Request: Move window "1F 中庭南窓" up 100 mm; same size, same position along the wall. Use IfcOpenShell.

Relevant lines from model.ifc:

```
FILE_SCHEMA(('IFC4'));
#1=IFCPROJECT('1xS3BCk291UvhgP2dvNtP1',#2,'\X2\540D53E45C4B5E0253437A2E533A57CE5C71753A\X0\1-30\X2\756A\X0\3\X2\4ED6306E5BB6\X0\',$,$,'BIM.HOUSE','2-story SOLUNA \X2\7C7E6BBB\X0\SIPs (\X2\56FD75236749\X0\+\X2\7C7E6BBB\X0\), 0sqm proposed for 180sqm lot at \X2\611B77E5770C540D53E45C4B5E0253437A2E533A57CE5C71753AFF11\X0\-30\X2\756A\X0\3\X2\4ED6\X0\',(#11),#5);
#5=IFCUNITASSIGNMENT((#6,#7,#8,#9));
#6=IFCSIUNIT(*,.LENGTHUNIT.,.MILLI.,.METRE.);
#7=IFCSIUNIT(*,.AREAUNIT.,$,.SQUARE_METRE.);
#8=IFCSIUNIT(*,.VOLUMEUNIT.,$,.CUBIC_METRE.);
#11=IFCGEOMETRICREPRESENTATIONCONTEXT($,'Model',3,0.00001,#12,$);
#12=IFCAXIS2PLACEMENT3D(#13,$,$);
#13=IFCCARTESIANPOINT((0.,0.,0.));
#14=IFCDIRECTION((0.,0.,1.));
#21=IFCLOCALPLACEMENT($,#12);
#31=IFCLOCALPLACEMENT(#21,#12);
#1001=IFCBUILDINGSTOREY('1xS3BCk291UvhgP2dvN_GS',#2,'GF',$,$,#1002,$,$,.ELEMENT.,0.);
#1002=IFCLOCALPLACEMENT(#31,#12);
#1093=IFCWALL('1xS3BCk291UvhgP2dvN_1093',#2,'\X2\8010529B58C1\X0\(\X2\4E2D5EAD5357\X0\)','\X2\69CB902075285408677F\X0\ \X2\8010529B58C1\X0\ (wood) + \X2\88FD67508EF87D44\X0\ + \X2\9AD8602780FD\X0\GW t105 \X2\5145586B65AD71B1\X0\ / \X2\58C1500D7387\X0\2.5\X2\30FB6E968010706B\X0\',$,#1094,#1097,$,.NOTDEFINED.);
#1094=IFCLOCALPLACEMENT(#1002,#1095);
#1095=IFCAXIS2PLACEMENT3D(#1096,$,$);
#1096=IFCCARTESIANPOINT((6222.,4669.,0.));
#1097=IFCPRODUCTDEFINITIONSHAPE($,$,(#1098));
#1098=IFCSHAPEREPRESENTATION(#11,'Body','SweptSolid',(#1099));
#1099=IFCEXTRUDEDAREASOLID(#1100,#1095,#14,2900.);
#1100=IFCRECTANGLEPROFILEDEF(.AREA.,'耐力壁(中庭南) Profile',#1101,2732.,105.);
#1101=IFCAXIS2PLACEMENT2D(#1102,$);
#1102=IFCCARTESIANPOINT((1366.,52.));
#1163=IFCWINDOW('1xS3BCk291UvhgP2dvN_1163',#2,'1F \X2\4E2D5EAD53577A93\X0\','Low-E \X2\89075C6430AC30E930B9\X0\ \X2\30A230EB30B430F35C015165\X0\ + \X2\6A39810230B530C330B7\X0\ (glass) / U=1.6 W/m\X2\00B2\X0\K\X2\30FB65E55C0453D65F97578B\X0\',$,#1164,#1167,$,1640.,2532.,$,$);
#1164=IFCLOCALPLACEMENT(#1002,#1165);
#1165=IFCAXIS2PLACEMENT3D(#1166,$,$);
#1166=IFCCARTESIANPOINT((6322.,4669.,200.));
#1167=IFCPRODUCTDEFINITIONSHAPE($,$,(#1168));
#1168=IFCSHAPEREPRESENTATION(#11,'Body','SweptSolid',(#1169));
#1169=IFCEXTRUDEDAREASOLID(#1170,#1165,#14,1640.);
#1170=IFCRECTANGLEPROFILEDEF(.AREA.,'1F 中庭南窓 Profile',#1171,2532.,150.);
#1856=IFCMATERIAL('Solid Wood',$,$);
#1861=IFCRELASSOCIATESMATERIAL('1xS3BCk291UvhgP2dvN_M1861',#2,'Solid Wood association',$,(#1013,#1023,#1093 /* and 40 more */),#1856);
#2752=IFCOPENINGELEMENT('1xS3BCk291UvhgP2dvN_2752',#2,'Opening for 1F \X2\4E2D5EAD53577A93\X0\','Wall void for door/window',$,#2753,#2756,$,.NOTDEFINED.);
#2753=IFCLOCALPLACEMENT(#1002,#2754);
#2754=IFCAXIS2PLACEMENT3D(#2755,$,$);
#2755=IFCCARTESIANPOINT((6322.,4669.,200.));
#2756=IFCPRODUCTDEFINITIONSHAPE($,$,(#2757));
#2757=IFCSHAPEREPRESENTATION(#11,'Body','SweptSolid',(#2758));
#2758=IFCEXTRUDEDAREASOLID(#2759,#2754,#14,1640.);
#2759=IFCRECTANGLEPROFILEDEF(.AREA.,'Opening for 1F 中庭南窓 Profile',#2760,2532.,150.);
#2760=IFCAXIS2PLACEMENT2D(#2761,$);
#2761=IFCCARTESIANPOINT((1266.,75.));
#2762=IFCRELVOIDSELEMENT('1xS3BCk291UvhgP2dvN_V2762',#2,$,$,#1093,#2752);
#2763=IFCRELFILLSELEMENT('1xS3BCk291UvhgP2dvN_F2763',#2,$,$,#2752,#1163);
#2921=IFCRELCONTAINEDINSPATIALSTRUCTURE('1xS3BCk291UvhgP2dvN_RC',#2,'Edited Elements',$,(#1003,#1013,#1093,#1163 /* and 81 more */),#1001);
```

```python
import numpy as np
import ifcopenshell
import ifcopenshell.api.geometry
import ifcopenshell.util.placement
import ifcopenshell.util.unit

model = ifcopenshell.open("model.ifc")
unit_scale = ifcopenshell.util.unit.calculate_unit_scale(model)

window = model.by_id(1163)
opening = window.FillsVoids[0].RelatingOpeningElement
dz = 100.0

shift = np.array([0.0, 0.0, dz])
# The window is not placed relative to its opening, so move both.
for product in (opening, window):
    matrix = ifcopenshell.util.placement.get_local_placement(product.ObjectPlacement)
    matrix[:3, 3] += shift
    ifcopenshell.api.geometry.edit_object_placement(model, product=product, matrix=matrix, is_si=False)

print(f"moved by {dz * unit_scale:+.3f} m")

model.write("model-out.ifc")
```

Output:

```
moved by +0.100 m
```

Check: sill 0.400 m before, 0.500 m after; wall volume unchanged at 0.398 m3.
